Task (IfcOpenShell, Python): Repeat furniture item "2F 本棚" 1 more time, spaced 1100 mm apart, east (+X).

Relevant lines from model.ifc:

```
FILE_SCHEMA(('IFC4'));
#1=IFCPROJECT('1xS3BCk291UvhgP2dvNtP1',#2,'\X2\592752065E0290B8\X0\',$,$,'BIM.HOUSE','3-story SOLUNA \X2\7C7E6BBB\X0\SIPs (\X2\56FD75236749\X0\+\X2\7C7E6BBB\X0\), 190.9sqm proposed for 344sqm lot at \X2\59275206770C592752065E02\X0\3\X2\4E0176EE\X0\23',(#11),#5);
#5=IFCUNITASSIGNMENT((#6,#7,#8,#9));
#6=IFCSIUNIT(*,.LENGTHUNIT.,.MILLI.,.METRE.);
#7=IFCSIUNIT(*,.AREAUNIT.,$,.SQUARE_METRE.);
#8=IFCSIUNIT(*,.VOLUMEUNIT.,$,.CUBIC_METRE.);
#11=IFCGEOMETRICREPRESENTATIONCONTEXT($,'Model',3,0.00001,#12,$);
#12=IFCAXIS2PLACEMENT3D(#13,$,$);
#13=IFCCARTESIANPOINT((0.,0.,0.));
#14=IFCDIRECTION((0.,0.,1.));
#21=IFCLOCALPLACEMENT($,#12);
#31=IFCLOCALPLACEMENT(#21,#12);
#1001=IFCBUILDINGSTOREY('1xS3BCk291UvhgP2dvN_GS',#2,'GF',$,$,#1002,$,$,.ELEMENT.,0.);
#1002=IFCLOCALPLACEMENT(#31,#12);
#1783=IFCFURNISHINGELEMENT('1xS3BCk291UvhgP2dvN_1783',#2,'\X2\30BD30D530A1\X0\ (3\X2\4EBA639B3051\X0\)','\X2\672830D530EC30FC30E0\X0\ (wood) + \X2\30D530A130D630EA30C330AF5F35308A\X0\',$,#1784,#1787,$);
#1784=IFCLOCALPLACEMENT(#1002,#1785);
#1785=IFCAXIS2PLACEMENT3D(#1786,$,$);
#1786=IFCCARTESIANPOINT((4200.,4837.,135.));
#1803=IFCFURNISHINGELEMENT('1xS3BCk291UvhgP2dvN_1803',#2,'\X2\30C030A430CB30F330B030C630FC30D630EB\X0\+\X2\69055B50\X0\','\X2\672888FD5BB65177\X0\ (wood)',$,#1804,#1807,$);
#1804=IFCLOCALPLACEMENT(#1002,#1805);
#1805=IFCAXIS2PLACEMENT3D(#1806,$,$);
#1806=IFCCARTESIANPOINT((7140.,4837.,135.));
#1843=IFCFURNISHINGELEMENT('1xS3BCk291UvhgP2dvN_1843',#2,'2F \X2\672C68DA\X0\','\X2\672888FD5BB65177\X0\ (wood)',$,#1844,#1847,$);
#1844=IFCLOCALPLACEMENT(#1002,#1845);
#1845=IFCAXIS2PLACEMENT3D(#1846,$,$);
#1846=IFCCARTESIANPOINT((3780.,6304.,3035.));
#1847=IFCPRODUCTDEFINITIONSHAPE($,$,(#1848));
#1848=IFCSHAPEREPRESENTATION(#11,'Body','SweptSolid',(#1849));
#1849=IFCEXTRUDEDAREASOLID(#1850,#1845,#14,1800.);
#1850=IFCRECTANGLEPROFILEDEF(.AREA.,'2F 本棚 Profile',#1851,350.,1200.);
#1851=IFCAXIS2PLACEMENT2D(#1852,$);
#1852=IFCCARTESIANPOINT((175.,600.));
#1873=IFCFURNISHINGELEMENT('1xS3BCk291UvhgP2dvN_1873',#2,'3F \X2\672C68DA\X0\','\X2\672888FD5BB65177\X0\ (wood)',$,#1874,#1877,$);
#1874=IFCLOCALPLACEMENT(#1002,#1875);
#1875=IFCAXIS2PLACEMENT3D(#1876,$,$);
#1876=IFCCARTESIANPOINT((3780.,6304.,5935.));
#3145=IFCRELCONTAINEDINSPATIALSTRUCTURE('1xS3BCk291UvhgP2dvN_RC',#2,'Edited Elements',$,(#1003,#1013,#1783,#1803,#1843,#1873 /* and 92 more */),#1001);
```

```python
import numpy as np
import ifcopenshell
import ifcopenshell.api.geometry
import ifcopenshell.api.root
import ifcopenshell.util.element
import ifcopenshell.util.placement

model = ifcopenshell.open("model.ifc")


def reuse_history(source, copy):
    """copy_class also copies each property set's owner history, people and application; keep the originals."""
    for rel in copy.IsDefinedBy:
        if rel.is_a("IfcRelDefinesByProperties") and (history := rel.RelatingPropertyDefinition.OwnerHistory):
            rel.RelatingPropertyDefinition.OwnerHistory = source.OwnerHistory
            ifcopenshell.util.element.remove_deep2(model, history)


source = model.by_guid("1xS3BCk291UvhgP2dvN_1843")
base = ifcopenshell.util.placement.get_local_placement(source.ObjectPlacement)
step = np.array([1.0, 0.0, 0.0]) * 1100.0

for i in range(1, 2):
    copy = ifcopenshell.api.root.copy_class(model, product=source)
    copy.Representation = ifcopenshell.util.element.copy_deep(
        model, source.Representation, exclude=["IfcGeometricRepresentationContext", "IfcRepresentationMap"]
    )
    reuse_history(source, copy)
    matrix = base.copy()
    matrix[:3, 3] += i * step
    print("added at", matrix[:3, 3].round(3) + 0.0)
    ifcopenshell.api.geometry.edit_object_placement(model, product=copy, matrix=matrix, is_si=False)

model.write("model_rev.ifc")
```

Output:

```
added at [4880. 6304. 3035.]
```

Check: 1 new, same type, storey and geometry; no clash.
